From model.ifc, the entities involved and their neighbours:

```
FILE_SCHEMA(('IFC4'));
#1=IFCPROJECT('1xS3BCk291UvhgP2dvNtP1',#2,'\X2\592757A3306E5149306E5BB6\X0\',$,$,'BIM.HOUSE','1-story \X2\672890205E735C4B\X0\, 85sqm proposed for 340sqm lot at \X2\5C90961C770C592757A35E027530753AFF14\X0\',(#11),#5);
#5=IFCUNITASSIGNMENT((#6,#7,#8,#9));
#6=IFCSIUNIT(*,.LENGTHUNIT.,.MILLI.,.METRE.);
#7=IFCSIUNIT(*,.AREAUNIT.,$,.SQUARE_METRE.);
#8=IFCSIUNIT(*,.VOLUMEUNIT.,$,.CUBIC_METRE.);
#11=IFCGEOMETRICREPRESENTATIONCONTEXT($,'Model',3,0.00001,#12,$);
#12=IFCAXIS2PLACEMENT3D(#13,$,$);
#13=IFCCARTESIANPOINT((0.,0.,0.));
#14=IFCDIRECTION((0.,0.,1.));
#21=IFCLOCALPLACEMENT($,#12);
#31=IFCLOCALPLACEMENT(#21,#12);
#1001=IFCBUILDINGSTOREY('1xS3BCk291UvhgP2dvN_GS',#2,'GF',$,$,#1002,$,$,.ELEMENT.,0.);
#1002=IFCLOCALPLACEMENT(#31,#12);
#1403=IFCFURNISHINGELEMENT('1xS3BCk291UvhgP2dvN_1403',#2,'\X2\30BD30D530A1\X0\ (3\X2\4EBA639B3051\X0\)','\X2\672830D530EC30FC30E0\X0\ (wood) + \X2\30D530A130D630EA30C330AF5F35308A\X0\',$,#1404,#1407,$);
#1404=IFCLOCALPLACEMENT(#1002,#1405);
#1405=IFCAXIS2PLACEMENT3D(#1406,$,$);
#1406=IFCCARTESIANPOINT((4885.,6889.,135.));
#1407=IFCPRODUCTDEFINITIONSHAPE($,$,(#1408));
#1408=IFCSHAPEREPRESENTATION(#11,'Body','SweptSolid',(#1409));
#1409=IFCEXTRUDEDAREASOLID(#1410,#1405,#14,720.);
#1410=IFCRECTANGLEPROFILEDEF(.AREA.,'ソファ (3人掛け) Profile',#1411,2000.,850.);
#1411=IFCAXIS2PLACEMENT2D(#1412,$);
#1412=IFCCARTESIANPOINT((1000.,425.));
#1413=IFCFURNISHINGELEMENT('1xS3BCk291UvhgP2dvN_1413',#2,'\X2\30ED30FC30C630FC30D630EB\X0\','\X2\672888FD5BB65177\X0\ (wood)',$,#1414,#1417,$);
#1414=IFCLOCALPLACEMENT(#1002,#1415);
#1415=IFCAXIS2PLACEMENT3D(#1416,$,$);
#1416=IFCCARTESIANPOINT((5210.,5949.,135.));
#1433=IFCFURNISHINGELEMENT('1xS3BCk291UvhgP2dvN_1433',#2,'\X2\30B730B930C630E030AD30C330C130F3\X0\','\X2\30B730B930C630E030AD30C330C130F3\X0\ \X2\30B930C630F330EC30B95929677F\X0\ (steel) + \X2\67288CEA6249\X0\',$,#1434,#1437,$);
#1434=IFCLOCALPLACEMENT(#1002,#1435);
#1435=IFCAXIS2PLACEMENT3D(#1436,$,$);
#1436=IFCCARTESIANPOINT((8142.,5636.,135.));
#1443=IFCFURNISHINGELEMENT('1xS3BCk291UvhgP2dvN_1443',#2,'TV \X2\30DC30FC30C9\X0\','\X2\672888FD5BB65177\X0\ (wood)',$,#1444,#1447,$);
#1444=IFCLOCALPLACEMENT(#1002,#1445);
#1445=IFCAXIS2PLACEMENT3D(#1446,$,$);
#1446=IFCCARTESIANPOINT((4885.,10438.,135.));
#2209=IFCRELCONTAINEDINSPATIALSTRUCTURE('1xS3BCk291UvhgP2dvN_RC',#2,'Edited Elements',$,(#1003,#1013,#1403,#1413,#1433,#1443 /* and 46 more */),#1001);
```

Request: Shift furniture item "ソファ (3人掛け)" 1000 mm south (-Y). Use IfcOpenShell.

```python
import ifcopenshell
import ifcopenshell.api.geometry
import ifcopenshell.util.placement
import ifcopenshell.util.unit

model = ifcopenshell.open("model.ifc")
unit_scale = ifcopenshell.util.unit.calculate_unit_scale(model)

item = model.by_guid("1xS3BCk291UvhgP2dvN_1403")
matrix = ifcopenshell.util.placement.get_local_placement(item.ObjectPlacement)
matrix[1, 3] -= 1 / unit_scale
ifcopenshell.api.geometry.edit_object_placement(model, product=item, matrix=matrix, is_si=False)

print(ifcopenshell.util.placement.get_local_placement(item.ObjectPlacement).round(3) + 0.0)

model.write("model_updated.ifc")
```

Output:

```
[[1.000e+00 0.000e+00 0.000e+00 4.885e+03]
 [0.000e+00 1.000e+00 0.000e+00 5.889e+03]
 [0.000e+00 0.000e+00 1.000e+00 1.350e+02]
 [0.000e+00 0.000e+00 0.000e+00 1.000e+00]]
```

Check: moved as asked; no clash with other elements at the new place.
